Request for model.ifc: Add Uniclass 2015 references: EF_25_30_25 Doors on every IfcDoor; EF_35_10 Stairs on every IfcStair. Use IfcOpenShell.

First a look at what the model holds.

```python
import ifcopenshell

model = ifcopenshell.open("model.ifc")
print(model.schema)
print("classifications:", [c.Name for c in model.by_type("IfcClassification")])
for ifc_class in ("IfcDoor", "IfcRoof", "IfcStair", "IfcWall", "IfcWindow"):
    print(ifc_class, len(model.by_type(ifc_class)))
```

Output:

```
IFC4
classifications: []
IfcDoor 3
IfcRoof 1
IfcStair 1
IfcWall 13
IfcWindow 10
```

```python
import ifcopenshell
import ifcopenshell.api.classification

model = ifcopenshell.open("model.ifc")

system = ifcopenshell.api.classification.add_classification(model, classification="Uniclass 2015")

codes = {
    "IfcDoor": ("EF_25_30_25", "Doors"),
    "IfcStair": ("EF_35_10", "Stairs"),
}
for ifc_class, (code, name) in codes.items():
    products = model.by_type(ifc_class)
    ifcopenshell.api.classification.add_reference(
        model, products=products, classification=system, identification=code, name=name
    )
    print(code, len(products))

model.write("model_rev.ifc")
```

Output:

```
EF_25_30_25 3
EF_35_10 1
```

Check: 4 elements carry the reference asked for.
